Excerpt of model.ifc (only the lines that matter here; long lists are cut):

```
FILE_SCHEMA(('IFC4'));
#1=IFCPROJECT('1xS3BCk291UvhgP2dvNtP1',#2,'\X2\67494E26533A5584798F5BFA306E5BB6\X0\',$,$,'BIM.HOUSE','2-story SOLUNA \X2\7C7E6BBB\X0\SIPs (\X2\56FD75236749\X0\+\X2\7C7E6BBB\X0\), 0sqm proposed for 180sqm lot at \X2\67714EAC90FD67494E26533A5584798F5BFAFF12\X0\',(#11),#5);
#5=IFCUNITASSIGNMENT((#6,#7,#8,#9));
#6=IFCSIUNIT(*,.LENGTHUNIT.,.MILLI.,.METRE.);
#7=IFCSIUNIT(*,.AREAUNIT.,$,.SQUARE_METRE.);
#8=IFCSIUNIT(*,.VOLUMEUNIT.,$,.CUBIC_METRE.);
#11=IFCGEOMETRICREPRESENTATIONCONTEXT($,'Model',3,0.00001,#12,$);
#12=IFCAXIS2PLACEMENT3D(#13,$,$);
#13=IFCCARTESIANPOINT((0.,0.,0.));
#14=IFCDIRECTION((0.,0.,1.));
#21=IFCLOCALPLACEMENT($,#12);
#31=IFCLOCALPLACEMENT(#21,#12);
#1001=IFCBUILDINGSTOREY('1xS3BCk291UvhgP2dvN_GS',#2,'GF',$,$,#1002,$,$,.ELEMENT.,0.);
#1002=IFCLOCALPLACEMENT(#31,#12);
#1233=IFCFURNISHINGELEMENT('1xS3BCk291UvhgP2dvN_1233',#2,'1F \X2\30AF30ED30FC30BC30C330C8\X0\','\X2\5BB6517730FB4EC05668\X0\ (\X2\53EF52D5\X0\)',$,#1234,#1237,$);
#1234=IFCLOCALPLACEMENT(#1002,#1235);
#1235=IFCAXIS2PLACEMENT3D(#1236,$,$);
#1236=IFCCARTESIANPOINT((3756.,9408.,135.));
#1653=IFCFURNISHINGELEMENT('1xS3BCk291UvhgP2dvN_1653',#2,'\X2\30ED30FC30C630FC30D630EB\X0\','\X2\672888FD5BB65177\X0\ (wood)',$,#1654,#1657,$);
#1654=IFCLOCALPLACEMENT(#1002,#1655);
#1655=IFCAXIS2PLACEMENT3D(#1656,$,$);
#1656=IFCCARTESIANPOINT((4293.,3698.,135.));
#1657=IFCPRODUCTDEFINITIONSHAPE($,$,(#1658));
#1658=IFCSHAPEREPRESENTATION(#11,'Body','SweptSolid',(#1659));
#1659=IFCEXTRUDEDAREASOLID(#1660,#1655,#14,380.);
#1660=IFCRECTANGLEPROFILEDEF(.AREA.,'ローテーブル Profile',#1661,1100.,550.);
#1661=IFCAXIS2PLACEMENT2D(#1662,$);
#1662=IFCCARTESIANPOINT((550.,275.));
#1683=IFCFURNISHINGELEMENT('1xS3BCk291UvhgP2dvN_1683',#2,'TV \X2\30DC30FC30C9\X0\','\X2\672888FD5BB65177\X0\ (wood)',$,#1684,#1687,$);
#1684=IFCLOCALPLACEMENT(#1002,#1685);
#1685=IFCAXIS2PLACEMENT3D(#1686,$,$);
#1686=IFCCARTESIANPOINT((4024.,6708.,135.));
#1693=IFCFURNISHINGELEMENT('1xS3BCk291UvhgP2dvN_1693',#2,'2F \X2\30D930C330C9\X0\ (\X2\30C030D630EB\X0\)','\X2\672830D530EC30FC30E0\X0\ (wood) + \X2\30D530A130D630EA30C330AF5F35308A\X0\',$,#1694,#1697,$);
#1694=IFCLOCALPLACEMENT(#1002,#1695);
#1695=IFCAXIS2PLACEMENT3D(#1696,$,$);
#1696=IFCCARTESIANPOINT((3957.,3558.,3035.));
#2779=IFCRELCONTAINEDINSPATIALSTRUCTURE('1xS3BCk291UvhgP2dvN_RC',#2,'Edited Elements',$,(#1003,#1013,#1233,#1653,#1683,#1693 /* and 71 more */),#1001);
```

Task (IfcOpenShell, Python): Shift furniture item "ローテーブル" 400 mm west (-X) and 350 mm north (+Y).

```python
import ifcopenshell
import ifcopenshell.api.geometry
import ifcopenshell.util.placement
import ifcopenshell.util.unit

model = ifcopenshell.open("model.ifc")
unit_scale = ifcopenshell.util.unit.calculate_unit_scale(model)

item = model.by_guid("1xS3BCk291UvhgP2dvN_1653")
matrix = ifcopenshell.util.placement.get_local_placement(item.ObjectPlacement)
matrix[0, 3] -= 0.4 / unit_scale
matrix[1, 3] += 0.35 / unit_scale
ifcopenshell.api.geometry.edit_object_placement(model, product=item, matrix=matrix, is_si=False)

print(ifcopenshell.util.placement.get_local_placement(item.ObjectPlacement).round(3) + 0.0)

model.write("model_v2.ifc")
```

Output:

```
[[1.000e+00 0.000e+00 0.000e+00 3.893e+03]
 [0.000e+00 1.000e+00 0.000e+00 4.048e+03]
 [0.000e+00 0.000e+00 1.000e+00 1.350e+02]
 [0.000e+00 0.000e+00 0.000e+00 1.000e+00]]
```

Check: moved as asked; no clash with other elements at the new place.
